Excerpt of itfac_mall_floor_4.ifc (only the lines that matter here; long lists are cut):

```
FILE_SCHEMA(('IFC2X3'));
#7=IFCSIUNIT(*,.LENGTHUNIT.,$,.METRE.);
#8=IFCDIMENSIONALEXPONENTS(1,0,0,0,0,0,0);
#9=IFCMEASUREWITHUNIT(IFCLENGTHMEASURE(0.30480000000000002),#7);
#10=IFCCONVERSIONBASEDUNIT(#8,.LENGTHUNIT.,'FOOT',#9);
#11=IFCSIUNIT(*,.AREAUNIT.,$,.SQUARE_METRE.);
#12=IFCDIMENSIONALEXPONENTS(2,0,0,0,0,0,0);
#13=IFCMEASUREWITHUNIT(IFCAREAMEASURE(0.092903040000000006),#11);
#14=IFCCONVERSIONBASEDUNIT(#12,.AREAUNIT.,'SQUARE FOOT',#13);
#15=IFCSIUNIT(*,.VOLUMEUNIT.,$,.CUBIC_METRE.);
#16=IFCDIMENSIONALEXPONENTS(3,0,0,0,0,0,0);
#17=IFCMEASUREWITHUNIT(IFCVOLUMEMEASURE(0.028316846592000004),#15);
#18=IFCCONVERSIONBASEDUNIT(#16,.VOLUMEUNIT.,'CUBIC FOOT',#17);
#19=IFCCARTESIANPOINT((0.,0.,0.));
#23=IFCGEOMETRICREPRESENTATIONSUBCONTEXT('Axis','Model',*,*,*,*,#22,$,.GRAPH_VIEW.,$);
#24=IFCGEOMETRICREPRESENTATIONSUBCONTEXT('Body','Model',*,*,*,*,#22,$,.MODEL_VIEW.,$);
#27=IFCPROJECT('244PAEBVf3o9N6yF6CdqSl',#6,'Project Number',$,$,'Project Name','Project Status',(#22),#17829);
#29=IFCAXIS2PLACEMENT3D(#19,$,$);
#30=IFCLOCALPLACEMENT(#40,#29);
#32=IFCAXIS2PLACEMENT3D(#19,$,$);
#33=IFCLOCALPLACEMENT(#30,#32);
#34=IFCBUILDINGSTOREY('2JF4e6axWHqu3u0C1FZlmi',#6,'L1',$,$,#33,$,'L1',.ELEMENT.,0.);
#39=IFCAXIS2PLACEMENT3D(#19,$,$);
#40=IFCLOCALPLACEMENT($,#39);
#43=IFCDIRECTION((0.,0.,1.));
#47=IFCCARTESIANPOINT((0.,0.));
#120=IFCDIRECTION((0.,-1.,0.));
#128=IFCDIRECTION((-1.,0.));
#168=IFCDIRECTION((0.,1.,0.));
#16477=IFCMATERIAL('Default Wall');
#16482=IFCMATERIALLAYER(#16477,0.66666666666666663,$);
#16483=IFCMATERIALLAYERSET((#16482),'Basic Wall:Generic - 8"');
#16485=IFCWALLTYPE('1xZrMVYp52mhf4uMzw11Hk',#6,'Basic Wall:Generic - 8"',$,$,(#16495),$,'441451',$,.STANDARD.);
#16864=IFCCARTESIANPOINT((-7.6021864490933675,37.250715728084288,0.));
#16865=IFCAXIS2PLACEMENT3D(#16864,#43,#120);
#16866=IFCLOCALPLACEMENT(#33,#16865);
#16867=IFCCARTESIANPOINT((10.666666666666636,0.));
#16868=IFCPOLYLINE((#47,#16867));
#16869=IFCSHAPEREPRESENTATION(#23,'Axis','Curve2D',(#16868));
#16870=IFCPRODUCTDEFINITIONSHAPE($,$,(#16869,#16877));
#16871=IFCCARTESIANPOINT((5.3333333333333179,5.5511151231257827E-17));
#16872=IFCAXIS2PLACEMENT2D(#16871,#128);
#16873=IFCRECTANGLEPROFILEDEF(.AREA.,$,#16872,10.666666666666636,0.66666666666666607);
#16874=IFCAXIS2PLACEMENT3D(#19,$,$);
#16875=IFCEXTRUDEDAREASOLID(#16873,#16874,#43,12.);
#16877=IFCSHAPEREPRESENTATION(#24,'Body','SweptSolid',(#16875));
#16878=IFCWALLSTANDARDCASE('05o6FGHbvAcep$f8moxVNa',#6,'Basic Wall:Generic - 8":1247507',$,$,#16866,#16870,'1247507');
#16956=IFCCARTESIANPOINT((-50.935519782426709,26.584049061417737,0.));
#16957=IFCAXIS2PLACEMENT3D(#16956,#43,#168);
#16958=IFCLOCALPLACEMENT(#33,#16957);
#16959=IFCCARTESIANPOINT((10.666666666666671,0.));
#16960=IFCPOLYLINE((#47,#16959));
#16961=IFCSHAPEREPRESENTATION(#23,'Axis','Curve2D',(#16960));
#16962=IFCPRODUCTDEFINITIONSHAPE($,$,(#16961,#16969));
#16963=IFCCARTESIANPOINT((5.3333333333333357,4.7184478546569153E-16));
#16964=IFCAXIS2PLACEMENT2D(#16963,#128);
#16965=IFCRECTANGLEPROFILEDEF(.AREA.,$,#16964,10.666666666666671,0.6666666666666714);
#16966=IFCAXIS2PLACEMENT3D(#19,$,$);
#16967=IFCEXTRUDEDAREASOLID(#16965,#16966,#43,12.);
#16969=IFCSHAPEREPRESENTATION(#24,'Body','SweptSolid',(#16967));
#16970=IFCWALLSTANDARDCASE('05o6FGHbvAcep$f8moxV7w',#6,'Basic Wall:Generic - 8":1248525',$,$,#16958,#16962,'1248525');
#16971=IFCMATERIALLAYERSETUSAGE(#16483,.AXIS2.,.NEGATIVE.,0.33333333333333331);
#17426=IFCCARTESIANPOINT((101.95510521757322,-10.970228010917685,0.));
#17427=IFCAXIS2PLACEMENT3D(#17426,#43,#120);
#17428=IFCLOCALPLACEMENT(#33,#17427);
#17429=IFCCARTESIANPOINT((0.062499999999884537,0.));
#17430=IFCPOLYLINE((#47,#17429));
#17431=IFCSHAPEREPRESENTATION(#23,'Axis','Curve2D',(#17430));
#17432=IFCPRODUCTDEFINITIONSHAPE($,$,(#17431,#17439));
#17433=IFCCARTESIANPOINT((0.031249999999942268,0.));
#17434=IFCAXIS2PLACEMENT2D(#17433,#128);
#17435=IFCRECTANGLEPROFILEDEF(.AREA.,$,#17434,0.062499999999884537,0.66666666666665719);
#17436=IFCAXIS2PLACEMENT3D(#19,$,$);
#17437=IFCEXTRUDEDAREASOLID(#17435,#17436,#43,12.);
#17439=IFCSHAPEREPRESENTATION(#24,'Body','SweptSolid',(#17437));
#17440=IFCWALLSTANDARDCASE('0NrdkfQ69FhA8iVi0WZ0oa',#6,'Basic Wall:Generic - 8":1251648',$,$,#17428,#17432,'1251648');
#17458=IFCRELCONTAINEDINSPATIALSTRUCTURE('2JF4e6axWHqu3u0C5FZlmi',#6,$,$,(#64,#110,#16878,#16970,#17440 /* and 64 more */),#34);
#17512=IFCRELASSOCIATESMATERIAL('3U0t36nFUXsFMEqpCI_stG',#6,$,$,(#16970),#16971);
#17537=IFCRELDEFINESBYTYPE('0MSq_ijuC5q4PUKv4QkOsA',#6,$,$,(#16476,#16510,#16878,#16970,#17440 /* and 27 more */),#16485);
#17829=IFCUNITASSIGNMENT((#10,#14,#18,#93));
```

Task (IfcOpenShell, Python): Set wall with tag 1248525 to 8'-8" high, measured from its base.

```python
import ifcopenshell
import ifcopenshell.geom
import ifcopenshell.util.representation
import ifcopenshell.util.shape
import ifcopenshell.util.unit

model = ifcopenshell.open("itfac_mall_floor_4.ifc")
unit_scale = ifcopenshell.util.unit.calculate_unit_scale(model)
settings = ifcopenshell.geom.settings()


def volume(element):
    """Net volume in cubic metres, openings subtracted."""
    shape = ifcopenshell.geom.create_shape(settings, element)
    return ifcopenshell.util.shape.get_volume(shape.geometry)


wall = model.by_guid("05o6FGHbvAcep$f8moxV7w")
before = volume(wall)

body = ifcopenshell.util.representation.get_representation(wall, "Model", "Body")
solid = body.Items[0]
old_height = solid.Depth
solid.Depth = 104 * 0.0254 / unit_scale
after = volume(wall)

print(f"height {old_height:g} -> {solid.Depth:g}, volume {before:.3f} -> {after:.3f} m3")

model.write("itfac_mall_floor_4-out.ifc")
```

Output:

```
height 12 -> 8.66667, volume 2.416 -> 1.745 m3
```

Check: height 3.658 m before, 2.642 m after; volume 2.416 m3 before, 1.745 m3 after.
